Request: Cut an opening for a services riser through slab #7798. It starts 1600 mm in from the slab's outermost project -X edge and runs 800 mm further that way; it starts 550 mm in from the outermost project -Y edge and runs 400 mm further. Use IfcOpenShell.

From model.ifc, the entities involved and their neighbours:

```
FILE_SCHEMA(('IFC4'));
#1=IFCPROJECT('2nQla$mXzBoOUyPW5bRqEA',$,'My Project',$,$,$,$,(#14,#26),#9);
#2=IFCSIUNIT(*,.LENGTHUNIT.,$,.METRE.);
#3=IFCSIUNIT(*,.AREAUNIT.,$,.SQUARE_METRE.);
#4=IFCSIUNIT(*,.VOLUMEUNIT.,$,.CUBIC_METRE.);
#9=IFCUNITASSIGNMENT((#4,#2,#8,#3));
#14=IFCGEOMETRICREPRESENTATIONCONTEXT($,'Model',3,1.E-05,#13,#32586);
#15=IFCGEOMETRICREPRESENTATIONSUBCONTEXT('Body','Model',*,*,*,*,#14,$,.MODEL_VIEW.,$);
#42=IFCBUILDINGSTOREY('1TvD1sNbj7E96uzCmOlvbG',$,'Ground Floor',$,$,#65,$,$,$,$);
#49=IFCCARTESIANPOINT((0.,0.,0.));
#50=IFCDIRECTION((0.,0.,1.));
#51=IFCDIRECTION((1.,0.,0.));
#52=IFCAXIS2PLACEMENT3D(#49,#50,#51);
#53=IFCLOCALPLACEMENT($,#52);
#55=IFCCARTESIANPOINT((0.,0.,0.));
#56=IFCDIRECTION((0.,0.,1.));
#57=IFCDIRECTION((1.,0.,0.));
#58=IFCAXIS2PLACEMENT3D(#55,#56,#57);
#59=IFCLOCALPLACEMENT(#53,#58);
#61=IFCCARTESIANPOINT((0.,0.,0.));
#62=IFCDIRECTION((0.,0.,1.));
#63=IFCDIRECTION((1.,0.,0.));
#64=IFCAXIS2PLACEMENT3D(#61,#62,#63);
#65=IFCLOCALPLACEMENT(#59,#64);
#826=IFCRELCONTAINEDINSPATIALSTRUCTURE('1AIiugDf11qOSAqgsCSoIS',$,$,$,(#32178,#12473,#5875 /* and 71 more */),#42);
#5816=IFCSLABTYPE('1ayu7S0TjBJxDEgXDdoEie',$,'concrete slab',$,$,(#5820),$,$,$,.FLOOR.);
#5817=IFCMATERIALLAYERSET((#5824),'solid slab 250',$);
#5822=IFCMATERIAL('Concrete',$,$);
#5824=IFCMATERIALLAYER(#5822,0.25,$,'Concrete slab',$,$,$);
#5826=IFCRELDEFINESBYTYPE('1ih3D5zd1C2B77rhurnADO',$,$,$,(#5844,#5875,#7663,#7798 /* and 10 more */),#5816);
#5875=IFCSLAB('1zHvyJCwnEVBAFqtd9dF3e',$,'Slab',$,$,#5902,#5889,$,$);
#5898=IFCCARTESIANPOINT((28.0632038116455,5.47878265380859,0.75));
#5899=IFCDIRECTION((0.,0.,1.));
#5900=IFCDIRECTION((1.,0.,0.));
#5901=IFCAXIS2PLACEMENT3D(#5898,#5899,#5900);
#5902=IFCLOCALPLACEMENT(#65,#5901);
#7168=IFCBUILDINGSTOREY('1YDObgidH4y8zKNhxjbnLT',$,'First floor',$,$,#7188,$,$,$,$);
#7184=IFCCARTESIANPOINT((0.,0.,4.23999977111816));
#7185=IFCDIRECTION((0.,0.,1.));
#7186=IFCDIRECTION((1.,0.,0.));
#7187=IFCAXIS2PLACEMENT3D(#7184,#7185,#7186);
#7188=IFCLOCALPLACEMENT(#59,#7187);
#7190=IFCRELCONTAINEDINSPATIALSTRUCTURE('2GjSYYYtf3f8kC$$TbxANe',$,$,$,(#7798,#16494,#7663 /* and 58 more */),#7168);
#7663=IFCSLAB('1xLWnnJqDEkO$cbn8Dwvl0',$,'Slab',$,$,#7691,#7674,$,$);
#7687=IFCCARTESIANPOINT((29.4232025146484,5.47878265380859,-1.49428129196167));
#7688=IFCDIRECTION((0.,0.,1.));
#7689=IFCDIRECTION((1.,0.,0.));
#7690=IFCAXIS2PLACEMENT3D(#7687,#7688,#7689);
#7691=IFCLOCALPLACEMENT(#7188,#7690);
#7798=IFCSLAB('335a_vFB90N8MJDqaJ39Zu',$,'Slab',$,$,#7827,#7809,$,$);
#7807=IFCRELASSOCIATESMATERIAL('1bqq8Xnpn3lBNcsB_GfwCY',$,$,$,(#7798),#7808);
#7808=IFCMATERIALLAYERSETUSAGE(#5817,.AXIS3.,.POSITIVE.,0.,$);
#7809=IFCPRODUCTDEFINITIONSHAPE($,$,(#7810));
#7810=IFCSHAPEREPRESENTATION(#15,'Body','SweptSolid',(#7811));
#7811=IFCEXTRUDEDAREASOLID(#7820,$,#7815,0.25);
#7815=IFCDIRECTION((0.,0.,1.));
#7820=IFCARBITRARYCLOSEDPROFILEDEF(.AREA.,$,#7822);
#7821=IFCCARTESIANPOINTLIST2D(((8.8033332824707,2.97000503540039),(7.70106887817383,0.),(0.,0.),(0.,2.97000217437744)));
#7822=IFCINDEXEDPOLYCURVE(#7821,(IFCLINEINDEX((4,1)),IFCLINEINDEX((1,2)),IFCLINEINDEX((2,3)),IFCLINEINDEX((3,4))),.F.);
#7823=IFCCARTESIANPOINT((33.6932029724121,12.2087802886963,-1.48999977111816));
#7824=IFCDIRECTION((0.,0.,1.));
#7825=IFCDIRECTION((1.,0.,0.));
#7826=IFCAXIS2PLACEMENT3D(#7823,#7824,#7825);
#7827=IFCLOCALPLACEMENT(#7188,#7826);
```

```python
import numpy as np
import ifcopenshell
import ifcopenshell.api.feature
import ifcopenshell.api.geometry
import ifcopenshell.api.root
import ifcopenshell.geom
import ifcopenshell.util.placement
import ifcopenshell.util.representation
import ifcopenshell.util.shape
import ifcopenshell.util.unit

model = ifcopenshell.open("model.ifc")
unit_scale = ifcopenshell.util.unit.calculate_unit_scale(model)
settings = ifcopenshell.geom.settings()


def volume(element):
    """Net volume in cubic metres, openings subtracted."""
    shape = ifcopenshell.geom.create_shape(settings, element)
    return ifcopenshell.util.shape.get_volume(shape.geometry)


slab = model.by_guid("335a_vFB90N8MJDqaJ39Zu")
before = volume(slab)

# Extent in the slab's own axes, in metres. The edges named are its -X and -Y sides.
slab_shape = ifcopenshell.geom.create_shape(settings, slab)
vertices = ifcopenshell.util.shape.get_vertices(slab_shape.geometry)
x_min, y_min, bottom = vertices.min(axis=0)
top = vertices[:, 2].max()

opening = ifcopenshell.api.root.create_entity(model, ifc_class="IfcOpeningElement", name="Services riser opening", predefined_type="OPENING")
context = ifcopenshell.util.representation.get_context(model, "Model", "Body", "MODEL_VIEW")
width, depth = 0.8, 0.4
outline = [(0.0, 0.0), (width, 0.0), (width, depth), (0.0, depth), (0.0, 0.0)]
# Overshoot both faces by 50 mm so the cut is clean.
shape = ifcopenshell.api.geometry.add_slab_representation(
    model, context=context, depth=top - bottom + 0.1, polyline=outline
)
ifcopenshell.api.geometry.assign_representation(model, product=opening, representation=shape)

matrix = ifcopenshell.util.placement.get_local_placement(slab.ObjectPlacement)
matrix[:, 3] = matrix @ np.append(np.array([x_min + 1.6, y_min + 0.55, bottom - 0.05]) / unit_scale, 1.0)
ifcopenshell.api.geometry.edit_object_placement(model, product=opening, matrix=matrix, is_si=False)
ifcopenshell.api.feature.add_feature(model, feature=opening, element=slab)

after = volume(slab)

print(f"slab volume {before:.3f} -> {after:.3f} m3")

model.write("model_v2.ifc")
```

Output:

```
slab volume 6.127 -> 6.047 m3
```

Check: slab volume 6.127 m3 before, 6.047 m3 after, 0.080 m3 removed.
